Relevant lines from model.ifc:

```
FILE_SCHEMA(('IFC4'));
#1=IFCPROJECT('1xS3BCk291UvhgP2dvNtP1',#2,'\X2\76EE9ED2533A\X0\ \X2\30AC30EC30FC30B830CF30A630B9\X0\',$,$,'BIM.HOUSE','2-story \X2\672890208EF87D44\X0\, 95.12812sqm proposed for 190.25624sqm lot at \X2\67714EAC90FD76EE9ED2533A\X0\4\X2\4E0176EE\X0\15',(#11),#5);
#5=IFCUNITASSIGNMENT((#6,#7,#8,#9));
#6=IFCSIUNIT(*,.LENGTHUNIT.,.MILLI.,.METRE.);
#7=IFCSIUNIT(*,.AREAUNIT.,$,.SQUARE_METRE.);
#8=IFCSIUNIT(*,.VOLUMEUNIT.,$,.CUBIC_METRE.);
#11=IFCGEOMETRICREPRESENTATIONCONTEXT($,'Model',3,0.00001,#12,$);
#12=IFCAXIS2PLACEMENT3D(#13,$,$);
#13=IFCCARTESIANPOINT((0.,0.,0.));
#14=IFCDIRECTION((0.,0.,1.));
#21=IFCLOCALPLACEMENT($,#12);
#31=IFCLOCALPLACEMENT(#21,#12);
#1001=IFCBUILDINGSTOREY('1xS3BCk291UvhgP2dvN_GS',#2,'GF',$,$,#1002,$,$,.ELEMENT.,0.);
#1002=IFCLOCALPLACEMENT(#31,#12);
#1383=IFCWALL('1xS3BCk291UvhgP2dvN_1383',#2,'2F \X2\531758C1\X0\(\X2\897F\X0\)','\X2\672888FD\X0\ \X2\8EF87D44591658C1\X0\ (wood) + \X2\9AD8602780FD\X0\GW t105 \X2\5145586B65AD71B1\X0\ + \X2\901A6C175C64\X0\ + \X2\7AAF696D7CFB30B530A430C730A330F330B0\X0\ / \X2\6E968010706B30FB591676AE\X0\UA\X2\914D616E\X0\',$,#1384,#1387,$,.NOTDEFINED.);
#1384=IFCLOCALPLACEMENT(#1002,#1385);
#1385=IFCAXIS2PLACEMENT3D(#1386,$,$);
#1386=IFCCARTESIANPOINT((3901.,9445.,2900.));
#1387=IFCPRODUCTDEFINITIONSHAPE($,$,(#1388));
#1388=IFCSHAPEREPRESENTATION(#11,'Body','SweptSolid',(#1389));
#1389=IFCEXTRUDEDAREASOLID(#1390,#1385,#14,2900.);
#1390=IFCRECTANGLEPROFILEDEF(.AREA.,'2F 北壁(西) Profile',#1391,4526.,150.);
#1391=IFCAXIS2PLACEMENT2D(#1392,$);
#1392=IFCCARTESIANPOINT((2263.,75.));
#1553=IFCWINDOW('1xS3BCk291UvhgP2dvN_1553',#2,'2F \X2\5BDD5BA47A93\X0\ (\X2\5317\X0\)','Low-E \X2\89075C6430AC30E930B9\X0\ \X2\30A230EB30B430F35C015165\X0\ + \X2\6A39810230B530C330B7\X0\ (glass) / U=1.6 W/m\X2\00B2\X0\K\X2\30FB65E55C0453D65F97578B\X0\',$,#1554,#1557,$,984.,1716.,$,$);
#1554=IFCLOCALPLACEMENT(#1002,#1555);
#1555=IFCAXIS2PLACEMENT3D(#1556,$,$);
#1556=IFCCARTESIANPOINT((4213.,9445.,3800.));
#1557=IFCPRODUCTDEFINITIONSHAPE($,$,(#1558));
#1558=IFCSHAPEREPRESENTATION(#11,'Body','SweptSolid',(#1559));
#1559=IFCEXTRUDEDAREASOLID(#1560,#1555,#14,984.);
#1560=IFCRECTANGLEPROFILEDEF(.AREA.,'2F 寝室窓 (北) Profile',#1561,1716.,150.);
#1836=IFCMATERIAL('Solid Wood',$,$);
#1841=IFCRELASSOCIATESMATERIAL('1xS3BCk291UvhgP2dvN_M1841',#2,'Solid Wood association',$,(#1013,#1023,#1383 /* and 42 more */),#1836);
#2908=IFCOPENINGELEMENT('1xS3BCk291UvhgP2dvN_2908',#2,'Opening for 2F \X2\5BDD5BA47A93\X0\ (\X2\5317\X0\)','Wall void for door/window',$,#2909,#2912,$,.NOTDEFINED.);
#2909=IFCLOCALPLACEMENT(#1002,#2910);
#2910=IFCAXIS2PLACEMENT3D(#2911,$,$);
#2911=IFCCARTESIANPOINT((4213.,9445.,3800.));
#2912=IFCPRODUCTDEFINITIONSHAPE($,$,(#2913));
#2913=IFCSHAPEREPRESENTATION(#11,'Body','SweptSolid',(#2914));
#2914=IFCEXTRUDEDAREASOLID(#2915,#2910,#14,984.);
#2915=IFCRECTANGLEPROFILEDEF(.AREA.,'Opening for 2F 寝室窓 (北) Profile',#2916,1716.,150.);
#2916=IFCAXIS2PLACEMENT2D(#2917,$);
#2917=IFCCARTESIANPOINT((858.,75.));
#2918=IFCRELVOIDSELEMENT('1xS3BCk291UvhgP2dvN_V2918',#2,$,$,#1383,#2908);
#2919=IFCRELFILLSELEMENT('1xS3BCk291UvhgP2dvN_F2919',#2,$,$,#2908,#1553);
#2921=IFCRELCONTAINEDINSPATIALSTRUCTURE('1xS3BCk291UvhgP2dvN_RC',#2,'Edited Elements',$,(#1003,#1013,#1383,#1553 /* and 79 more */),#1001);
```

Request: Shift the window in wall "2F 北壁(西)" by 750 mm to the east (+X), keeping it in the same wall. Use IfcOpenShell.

```python
import ifcopenshell
import ifcopenshell.api.geometry
import ifcopenshell.util.placement
import ifcopenshell.util.unit

model = ifcopenshell.open("model.ifc")
unit_scale = ifcopenshell.util.unit.calculate_unit_scale(model)

window = model.by_id(1553)
opening = window.FillsVoids[0].RelatingOpeningElement
wall = opening.VoidsElements[0].RelatingBuildingElement

wall_matrix = ifcopenshell.util.placement.get_local_placement(wall.ObjectPlacement)
shift = wall_matrix[:3, 0] * 0.75 / unit_scale
before = ifcopenshell.util.placement.get_local_placement(window.ObjectPlacement)[:3, 3].copy()

# The window is not placed relative to its opening, so move both.
for product in (opening, window):
    matrix = ifcopenshell.util.placement.get_local_placement(product.ObjectPlacement)
    matrix[:3, 3] += shift
    ifcopenshell.api.geometry.edit_object_placement(model, product=product, matrix=matrix, is_si=False)

after = ifcopenshell.util.placement.get_local_placement(window.ObjectPlacement)[:3, 3]
print("window moved by", (after - before).round(3) + 0.0)

model.write("model-out.ifc")
```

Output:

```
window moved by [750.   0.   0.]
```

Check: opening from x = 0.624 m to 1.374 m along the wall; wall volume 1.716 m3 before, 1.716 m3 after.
